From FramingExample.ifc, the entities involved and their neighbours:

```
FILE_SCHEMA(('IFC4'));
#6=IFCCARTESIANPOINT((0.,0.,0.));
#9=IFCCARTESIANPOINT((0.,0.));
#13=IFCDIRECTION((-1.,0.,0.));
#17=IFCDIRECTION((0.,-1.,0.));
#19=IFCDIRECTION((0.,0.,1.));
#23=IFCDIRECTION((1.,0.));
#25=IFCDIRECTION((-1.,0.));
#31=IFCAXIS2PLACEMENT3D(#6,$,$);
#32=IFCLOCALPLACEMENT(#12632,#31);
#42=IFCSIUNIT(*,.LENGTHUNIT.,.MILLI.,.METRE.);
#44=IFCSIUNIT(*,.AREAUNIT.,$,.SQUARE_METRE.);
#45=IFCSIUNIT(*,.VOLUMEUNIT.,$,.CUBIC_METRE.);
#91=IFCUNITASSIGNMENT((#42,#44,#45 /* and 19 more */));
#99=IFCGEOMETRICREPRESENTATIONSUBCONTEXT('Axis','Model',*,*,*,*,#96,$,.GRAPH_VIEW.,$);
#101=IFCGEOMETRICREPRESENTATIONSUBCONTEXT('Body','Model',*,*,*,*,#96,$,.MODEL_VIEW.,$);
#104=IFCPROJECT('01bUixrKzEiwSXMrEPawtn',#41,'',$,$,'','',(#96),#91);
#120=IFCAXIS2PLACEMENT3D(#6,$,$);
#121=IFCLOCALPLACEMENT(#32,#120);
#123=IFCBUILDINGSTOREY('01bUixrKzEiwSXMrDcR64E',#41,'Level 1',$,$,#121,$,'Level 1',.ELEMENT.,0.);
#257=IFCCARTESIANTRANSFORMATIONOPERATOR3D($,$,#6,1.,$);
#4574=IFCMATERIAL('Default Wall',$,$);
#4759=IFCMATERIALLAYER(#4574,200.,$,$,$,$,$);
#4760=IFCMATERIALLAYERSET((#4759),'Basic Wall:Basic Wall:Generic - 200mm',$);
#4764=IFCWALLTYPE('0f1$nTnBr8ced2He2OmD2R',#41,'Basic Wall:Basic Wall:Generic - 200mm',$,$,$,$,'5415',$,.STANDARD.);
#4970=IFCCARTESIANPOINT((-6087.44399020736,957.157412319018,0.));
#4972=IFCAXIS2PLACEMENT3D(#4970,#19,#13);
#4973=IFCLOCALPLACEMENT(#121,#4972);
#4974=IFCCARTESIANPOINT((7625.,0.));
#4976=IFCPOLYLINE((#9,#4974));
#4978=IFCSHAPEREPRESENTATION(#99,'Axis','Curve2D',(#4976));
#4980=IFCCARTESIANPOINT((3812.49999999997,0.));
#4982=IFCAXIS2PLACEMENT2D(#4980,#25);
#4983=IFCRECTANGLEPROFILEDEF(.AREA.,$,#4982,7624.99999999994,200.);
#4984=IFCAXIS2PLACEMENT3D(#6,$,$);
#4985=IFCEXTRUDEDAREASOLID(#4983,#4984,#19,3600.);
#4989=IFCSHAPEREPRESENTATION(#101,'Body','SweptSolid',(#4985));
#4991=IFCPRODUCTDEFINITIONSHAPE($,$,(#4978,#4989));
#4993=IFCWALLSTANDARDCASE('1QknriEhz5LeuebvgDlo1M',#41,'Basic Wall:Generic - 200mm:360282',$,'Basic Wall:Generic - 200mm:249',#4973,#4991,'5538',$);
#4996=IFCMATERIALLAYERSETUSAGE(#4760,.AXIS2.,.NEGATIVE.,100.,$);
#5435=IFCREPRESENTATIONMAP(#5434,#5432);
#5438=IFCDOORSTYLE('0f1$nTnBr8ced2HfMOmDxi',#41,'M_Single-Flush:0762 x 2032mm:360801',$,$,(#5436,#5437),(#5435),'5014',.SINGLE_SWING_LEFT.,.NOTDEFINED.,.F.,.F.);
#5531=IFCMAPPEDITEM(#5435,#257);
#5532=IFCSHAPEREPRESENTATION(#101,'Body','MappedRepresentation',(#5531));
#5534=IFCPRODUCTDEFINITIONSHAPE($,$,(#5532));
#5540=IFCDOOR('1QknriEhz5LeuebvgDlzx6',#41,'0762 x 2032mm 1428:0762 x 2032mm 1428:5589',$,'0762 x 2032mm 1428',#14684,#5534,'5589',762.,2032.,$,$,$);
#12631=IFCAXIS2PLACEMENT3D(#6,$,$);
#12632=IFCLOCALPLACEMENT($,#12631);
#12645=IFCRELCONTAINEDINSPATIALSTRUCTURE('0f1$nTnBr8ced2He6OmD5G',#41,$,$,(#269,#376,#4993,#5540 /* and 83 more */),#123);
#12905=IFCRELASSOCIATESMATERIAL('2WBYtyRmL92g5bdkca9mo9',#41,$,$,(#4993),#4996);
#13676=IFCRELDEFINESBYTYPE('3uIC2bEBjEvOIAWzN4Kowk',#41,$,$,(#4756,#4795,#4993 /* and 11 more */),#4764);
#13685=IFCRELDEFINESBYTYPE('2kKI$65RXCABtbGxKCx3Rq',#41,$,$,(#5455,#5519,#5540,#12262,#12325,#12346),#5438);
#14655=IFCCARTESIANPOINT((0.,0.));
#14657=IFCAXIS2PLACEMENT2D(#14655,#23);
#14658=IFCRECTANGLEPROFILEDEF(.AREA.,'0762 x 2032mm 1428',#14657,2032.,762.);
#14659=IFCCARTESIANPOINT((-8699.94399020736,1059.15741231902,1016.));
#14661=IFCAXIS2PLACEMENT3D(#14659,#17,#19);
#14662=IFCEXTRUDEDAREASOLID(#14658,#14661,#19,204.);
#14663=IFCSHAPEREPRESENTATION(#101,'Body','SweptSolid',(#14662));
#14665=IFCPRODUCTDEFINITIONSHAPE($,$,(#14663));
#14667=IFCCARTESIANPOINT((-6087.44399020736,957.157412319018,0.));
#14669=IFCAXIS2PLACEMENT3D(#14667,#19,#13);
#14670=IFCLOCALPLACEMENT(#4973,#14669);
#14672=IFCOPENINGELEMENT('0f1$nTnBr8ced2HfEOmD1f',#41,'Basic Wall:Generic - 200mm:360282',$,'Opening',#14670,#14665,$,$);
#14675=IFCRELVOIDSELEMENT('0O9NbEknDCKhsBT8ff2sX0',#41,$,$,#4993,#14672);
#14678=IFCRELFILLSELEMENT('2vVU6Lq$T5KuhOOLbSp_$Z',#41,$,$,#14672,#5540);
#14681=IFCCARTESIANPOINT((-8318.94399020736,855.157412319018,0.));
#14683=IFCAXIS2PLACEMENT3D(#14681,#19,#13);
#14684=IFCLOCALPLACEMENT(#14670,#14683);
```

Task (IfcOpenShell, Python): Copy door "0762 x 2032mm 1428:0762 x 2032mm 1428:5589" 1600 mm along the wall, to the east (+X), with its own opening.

```python
import ifcopenshell
import ifcopenshell.api.feature
import ifcopenshell.api.geometry
import ifcopenshell.api.root
import ifcopenshell.geom
import ifcopenshell.util.element
import ifcopenshell.util.placement
import ifcopenshell.util.shape

model = ifcopenshell.open("FramingExample.ifc")
settings = ifcopenshell.geom.settings()


def volume(element):
    """Net volume in cubic metres, openings subtracted."""
    shape = ifcopenshell.geom.create_shape(settings, element)
    return ifcopenshell.util.shape.get_volume(shape.geometry)


def reuse_history(source, copy):
    """copy_class also copies each property set's owner history, people and application; keep the originals."""
    for rel in copy.IsDefinedBy:
        if rel.is_a("IfcRelDefinesByProperties") and (history := rel.RelatingPropertyDefinition.OwnerHistory):
            rel.RelatingPropertyDefinition.OwnerHistory = source.OwnerHistory
            ifcopenshell.util.element.remove_deep2(model, history)


door = model.by_guid("1QknriEhz5LeuebvgDlzx6")
opening = door.FillsVoids[0].RelatingOpeningElement
wall = opening.VoidsElements[0].RelatingBuildingElement
before = volume(wall)
shift = ifcopenshell.util.placement.get_local_placement(wall.ObjectPlacement)[:3, 0] * -1600.0

# copy_class copies the void relationship, type, container and properties, but no geometry.
new_opening = ifcopenshell.api.root.copy_class(model, product=opening)
new_opening.Representation = ifcopenshell.util.element.copy_deep(
    model, opening.Representation, exclude=["IfcGeometricRepresentationContext", "IfcRepresentationMap"]
)
new_opening.Name = "Basic Wall:Generic - 200mm"
new_door = ifcopenshell.api.root.copy_class(model, product=door)
new_door.Representation = ifcopenshell.util.element.copy_deep(
    model, door.Representation, exclude=["IfcGeometricRepresentationContext", "IfcRepresentationMap"]
)
new_door.Name = "0762 x 2032mm 1428:0762 x 2032mm 1428"
new_door.Tag = None
reuse_history(door, new_door)
ifcopenshell.api.feature.add_filling(model, opening=new_opening, element=new_door)

for old, new in ((opening, new_opening), (door, new_door)):
    matrix = ifcopenshell.util.placement.get_local_placement(old.ObjectPlacement)
    matrix[:3, 3] += shift
    ifcopenshell.api.geometry.edit_object_placement(model, product=new, matrix=matrix, is_si=False)

after = volume(wall)

print(f"wall volume {before:.3f} -> {after:.3f} m3")

model.write("FramingExample_rev.ifc")
```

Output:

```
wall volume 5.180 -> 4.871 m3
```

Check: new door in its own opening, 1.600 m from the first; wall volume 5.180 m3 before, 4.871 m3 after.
